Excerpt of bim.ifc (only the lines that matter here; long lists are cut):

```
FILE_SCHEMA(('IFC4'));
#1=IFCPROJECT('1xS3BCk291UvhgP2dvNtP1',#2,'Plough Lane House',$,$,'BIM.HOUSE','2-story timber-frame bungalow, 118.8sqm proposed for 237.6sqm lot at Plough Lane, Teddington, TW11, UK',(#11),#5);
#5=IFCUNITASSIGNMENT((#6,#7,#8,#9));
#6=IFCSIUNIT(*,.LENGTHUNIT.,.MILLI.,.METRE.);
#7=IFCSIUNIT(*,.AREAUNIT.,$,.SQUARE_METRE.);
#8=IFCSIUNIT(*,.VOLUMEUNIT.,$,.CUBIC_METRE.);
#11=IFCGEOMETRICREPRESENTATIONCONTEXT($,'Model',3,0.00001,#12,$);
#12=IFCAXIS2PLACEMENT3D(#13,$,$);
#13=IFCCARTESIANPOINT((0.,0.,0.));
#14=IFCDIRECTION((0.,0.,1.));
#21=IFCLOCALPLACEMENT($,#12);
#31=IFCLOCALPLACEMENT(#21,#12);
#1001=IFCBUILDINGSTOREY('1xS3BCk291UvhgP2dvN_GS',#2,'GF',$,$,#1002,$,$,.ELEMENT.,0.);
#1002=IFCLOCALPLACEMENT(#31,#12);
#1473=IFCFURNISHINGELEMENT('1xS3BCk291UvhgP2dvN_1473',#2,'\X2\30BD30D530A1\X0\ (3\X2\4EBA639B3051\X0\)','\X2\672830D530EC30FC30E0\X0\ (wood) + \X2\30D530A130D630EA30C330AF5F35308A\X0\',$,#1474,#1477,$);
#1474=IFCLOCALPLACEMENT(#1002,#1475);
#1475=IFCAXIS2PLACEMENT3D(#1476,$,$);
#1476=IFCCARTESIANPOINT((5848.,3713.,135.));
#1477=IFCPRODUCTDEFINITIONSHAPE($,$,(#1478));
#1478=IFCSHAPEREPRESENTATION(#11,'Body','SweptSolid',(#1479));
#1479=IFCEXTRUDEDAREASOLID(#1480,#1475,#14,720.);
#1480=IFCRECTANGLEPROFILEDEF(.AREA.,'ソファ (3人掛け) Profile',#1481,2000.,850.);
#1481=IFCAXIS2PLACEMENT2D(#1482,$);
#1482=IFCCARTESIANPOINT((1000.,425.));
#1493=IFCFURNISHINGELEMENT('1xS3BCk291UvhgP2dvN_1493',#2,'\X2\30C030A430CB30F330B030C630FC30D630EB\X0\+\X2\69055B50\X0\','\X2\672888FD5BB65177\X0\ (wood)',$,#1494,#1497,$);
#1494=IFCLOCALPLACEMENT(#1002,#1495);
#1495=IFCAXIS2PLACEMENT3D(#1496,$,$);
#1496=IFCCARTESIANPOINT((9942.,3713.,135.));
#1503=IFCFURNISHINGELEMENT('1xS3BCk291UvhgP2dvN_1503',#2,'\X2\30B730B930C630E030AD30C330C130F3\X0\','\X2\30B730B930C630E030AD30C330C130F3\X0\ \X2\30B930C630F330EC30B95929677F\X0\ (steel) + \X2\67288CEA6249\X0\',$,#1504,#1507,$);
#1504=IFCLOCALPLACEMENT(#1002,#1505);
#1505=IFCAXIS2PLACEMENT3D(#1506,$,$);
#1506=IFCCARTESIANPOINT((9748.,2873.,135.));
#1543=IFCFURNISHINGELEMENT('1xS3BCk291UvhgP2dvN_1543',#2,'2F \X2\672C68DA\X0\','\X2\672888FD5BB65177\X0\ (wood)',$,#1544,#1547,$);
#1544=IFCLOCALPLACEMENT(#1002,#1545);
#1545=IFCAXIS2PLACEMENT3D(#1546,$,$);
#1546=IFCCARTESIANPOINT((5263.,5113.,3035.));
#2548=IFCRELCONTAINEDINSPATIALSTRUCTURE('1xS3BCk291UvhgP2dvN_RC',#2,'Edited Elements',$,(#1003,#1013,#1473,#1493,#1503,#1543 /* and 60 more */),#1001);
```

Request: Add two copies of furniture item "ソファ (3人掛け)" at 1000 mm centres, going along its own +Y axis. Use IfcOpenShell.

```python
import ifcopenshell
import ifcopenshell.api.geometry
import ifcopenshell.api.root
import ifcopenshell.util.element
import ifcopenshell.util.placement
import ifcopenshell.util.unit

model = ifcopenshell.open("bim.ifc")
unit_scale = ifcopenshell.util.unit.calculate_unit_scale(model)


def reuse_history(source, copy):
    """copy_class also copies each property set's owner history, people and application; keep the originals."""
    for rel in copy.IsDefinedBy:
        if rel.is_a("IfcRelDefinesByProperties") and (history := rel.RelatingPropertyDefinition.OwnerHistory):
            rel.RelatingPropertyDefinition.OwnerHistory = source.OwnerHistory
            ifcopenshell.util.element.remove_deep2(model, history)


source = model.by_guid("1xS3BCk291UvhgP2dvN_1473")
base = ifcopenshell.util.placement.get_local_placement(source.ObjectPlacement)
step = base[:3, 1] * 1 / unit_scale

for i in range(1, 3):
    copy = ifcopenshell.api.root.copy_class(model, product=source)
    copy.Representation = ifcopenshell.util.element.copy_deep(
        model, source.Representation, exclude=["IfcGeometricRepresentationContext", "IfcRepresentationMap"]
    )
    reuse_history(source, copy)
    matrix = base.copy()
    matrix[:3, 3] += i * step
    print("added at", matrix[:3, 3].round(3) + 0.0)
    ifcopenshell.api.geometry.edit_object_placement(model, product=copy, matrix=matrix, is_si=False)

model.write("bim_edited.ifc")
```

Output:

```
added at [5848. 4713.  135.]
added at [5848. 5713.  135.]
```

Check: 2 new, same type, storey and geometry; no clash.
